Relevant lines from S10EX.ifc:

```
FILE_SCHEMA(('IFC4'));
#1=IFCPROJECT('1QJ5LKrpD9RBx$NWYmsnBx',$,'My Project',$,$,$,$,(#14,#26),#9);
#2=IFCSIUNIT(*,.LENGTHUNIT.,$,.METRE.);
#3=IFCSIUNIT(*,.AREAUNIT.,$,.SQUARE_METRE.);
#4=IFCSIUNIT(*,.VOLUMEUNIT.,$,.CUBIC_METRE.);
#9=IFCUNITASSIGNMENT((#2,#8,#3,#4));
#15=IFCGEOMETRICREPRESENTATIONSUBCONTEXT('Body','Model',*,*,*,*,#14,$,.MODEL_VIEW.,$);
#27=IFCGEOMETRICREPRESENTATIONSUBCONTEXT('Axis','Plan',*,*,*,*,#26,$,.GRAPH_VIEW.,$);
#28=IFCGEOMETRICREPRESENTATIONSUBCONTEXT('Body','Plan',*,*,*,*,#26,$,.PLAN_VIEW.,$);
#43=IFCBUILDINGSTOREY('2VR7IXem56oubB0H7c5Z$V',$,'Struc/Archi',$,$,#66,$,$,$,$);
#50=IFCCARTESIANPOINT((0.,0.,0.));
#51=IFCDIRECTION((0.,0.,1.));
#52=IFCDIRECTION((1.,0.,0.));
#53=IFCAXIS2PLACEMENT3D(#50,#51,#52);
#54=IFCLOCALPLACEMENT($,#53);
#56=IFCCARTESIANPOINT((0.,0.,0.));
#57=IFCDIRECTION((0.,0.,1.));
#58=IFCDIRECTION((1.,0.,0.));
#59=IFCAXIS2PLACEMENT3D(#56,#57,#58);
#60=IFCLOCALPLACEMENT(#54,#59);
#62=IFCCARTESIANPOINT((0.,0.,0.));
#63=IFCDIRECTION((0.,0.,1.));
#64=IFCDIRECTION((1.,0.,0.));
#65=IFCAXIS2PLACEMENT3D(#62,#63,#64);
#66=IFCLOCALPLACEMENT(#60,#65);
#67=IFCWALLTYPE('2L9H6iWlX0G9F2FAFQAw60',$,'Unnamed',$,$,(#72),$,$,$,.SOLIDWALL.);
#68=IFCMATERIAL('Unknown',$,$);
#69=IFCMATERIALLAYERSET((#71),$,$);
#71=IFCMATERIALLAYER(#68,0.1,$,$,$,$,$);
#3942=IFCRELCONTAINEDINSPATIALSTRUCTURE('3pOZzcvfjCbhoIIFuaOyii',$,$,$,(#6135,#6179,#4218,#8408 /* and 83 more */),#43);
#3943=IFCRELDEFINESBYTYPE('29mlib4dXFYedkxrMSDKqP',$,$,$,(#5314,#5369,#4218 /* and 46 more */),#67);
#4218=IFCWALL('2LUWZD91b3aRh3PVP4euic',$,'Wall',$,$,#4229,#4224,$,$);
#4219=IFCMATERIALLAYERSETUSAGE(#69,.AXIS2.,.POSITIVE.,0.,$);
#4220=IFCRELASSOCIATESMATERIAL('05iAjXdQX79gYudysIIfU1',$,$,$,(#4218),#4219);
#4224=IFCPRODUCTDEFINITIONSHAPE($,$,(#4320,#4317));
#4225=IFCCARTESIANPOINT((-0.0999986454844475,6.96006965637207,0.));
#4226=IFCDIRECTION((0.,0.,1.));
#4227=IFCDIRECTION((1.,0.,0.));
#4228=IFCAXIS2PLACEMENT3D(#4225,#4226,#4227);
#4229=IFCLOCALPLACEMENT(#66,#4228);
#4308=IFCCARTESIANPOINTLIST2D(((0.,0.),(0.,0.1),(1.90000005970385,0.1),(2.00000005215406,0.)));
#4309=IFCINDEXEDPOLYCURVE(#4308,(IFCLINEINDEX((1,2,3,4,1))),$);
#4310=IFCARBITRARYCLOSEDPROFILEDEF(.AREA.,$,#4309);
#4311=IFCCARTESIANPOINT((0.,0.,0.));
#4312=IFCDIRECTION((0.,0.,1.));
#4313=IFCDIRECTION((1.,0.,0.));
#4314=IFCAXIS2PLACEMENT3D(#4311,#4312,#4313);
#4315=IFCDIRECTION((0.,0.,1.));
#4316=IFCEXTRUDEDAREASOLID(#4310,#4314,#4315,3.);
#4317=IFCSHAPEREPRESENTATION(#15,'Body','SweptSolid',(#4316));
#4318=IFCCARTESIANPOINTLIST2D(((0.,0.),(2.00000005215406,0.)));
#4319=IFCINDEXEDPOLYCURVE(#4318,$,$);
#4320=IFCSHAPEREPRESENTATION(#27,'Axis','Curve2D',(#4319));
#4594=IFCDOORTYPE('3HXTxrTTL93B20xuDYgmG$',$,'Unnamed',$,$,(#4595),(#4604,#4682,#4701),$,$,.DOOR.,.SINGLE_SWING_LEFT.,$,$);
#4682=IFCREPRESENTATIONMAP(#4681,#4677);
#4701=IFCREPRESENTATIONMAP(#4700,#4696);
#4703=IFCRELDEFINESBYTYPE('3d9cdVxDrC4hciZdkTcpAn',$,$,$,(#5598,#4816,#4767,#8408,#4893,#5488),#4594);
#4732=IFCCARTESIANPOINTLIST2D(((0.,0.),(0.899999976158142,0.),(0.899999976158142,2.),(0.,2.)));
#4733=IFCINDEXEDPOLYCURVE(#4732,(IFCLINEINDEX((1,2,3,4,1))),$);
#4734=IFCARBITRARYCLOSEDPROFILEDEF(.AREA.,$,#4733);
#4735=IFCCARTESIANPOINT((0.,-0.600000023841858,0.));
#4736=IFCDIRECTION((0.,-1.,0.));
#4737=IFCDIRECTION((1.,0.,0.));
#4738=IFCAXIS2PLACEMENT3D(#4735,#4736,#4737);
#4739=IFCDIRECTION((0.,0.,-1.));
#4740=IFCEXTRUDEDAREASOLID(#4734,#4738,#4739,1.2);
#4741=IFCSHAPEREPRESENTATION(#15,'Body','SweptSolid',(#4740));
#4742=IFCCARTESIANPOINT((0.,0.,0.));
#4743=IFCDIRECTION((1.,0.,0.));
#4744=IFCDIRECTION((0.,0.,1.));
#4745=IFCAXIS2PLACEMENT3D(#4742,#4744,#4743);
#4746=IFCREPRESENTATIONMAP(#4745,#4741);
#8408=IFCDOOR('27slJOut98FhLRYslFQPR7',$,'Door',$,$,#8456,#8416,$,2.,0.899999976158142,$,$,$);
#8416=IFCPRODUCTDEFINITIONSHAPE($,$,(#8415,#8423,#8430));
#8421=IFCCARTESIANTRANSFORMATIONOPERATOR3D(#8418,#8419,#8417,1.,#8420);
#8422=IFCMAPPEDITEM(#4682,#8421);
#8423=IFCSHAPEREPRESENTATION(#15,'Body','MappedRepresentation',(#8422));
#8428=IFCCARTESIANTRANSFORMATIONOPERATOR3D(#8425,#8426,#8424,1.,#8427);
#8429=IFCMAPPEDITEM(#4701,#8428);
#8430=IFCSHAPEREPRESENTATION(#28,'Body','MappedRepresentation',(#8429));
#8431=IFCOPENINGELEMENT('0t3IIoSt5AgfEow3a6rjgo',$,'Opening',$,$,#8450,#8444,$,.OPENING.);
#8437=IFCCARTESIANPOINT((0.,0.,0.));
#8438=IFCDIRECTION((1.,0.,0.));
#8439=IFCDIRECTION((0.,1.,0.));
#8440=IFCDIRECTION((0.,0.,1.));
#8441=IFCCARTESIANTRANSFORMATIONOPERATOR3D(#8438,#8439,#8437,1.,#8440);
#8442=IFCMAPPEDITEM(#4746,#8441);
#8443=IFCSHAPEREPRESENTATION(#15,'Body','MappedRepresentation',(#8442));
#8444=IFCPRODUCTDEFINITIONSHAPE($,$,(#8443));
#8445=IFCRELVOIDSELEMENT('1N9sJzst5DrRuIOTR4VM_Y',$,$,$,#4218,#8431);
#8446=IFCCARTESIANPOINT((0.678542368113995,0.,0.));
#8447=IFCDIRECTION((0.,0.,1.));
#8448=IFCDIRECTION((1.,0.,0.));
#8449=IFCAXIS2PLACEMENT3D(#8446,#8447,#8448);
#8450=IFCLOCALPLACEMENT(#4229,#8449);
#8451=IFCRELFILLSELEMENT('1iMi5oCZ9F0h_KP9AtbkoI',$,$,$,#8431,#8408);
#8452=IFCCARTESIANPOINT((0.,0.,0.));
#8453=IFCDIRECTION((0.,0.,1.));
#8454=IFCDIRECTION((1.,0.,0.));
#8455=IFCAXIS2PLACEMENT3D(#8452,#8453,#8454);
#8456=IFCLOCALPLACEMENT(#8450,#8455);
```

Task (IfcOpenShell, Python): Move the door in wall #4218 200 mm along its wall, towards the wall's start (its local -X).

```python
import ifcopenshell
import ifcopenshell.api.geometry
import ifcopenshell.util.placement

model = ifcopenshell.open("S10EX.ifc")

door = model.by_guid("27slJOut98FhLRYslFQPR7")
opening = door.FillsVoids[0].RelatingOpeningElement
wall = opening.VoidsElements[0].RelatingBuildingElement

wall_matrix = ifcopenshell.util.placement.get_local_placement(wall.ObjectPlacement)
shift = wall_matrix[:3, 0] * -0.2
before = ifcopenshell.util.placement.get_local_placement(door.ObjectPlacement)[:3, 3].copy()

# The door is placed relative to its opening, so it follows when the opening moves.
matrix = ifcopenshell.util.placement.get_local_placement(opening.ObjectPlacement)
matrix[:3, 3] += shift
ifcopenshell.api.geometry.edit_object_placement(
    model, product=opening, matrix=matrix, is_si=False, should_transform_children=True
)

after = ifcopenshell.util.placement.get_local_placement(door.ObjectPlacement)[:3, 3]
print("door moved by", (after - before).round(3) + 0.0)

model.write("S10EX_rev.ifc")
```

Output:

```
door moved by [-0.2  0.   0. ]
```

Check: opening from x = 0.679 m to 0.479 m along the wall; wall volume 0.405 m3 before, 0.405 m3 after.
